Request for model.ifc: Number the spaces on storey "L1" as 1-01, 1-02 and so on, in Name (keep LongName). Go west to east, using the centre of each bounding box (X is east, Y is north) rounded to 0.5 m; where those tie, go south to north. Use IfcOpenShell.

First a look at what the model holds.

```python
import ifcopenshell
import ifcopenshell.util.element
import ifcopenshell.util.placement

model = ifcopenshell.open("model.ifc")
print(model.schema)
storey = next(s for s in model.by_type("IfcBuildingStorey") if s.Name == "L1")
spaces = [e for e in ifcopenshell.util.element.get_decomposition(storey) if e.is_a("IfcSpace")]
for e in sorted(spaces, key=lambda e: e.id()):
    origin = ifcopenshell.util.placement.get_local_placement(e.ObjectPlacement)[:3, 3]
    print(e.id(), e.Name, e.LongName, origin.round(2) + 0.0, sep=" | ")
```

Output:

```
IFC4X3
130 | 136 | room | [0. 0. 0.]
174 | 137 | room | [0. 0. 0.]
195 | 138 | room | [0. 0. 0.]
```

```python
import ifcopenshell
import ifcopenshell.geom
import ifcopenshell.util.element
import ifcopenshell.util.shape

model = ifcopenshell.open("model.ifc")
settings = ifcopenshell.geom.settings()
settings.set("use-world-coords", True)


def centre(element):
    shape = ifcopenshell.geom.create_shape(settings, element)
    return ifcopenshell.util.shape.get_bbox_centroid(shape.geometry)


storey = next(s for s in model.by_type("IfcBuildingStorey") if s.Name == "L1")
spaces = [e for e in ifcopenshell.util.element.get_decomposition(storey) if e.is_a("IfcSpace")]

# Insertion points can sit at a corner or the storey origin, so sort by the geometry (in metres).
centres = {e: centre(e) for e in spaces}
spaces.sort(key=lambda e: (round(centres[e][0] / 0.5), centres[e][1]))

for i, e in enumerate(spaces, start=1):
    number = f"1-{i:02d}"
    e.Name = number
    print(e.id(), number)

model.write("model-out.ifc")
```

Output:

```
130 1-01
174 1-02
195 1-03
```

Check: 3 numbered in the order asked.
